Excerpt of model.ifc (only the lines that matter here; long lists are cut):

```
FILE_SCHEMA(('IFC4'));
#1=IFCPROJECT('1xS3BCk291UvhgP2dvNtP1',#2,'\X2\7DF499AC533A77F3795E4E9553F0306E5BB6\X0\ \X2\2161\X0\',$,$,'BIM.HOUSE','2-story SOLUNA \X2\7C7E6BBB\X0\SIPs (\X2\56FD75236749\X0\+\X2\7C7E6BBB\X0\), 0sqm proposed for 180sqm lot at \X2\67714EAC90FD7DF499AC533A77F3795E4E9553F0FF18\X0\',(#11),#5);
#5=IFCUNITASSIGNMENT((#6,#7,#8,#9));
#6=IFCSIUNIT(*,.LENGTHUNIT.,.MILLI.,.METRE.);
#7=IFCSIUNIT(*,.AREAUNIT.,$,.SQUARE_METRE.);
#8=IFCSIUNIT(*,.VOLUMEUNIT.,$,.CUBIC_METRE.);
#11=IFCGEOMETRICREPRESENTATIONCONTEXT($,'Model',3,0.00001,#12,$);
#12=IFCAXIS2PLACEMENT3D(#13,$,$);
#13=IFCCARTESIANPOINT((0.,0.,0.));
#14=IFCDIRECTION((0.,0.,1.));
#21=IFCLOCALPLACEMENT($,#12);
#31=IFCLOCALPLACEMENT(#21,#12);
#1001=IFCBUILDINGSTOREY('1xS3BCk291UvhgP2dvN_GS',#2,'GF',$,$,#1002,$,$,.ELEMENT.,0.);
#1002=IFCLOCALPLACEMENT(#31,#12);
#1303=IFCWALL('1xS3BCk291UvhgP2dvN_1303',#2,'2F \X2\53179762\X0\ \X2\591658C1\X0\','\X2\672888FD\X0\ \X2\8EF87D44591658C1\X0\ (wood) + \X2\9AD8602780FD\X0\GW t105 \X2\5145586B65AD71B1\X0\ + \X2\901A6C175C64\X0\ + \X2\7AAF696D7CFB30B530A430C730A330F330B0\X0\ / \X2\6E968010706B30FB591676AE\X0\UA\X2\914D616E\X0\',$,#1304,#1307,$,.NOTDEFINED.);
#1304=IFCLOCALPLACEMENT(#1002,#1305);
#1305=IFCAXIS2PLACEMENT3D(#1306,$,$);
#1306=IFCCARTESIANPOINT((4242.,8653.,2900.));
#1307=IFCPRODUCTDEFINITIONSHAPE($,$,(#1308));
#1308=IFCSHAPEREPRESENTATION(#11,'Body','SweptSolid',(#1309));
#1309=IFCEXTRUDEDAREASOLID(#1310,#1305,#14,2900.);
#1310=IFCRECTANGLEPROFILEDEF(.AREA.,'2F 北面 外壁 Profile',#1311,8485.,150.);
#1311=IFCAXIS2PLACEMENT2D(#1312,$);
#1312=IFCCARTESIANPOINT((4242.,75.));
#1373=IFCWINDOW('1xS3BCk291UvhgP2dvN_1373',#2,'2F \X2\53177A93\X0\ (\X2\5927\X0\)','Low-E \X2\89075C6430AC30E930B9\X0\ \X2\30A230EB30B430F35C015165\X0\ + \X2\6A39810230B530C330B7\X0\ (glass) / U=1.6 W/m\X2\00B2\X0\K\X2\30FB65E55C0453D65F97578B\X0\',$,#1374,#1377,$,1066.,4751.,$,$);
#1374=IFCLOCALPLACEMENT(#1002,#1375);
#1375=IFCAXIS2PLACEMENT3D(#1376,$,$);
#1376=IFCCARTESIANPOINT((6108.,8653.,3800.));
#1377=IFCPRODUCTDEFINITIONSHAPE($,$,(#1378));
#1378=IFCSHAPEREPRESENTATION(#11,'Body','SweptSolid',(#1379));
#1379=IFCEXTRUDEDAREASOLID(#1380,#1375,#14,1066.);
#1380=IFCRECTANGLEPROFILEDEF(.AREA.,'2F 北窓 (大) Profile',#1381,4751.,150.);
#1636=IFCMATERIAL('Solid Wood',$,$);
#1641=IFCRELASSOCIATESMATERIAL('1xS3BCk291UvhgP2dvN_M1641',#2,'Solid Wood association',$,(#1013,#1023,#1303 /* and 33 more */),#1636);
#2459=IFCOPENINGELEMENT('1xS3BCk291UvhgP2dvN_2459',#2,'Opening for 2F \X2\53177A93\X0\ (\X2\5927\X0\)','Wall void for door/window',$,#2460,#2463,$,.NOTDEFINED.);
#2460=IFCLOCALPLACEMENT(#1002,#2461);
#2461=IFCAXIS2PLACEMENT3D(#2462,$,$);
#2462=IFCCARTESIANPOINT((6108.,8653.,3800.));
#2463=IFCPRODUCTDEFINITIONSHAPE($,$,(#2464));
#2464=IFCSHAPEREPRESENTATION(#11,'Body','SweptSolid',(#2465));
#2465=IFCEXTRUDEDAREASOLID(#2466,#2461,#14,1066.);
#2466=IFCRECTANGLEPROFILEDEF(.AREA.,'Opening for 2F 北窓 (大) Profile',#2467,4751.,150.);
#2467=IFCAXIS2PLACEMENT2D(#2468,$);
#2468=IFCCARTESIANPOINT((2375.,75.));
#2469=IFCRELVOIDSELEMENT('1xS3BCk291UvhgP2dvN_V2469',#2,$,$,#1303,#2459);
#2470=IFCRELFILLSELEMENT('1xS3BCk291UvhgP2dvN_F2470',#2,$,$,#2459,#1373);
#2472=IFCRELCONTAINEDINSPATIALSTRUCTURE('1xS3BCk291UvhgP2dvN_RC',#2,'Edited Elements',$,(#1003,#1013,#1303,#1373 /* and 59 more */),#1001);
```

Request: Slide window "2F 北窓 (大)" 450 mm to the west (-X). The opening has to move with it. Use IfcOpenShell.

```python
import ifcopenshell
import ifcopenshell.api.geometry
import ifcopenshell.util.placement
import ifcopenshell.util.unit

model = ifcopenshell.open("model.ifc")
unit_scale = ifcopenshell.util.unit.calculate_unit_scale(model)

window = model.by_guid("1xS3BCk291UvhgP2dvN_1373")
opening = window.FillsVoids[0].RelatingOpeningElement
wall = opening.VoidsElements[0].RelatingBuildingElement

wall_matrix = ifcopenshell.util.placement.get_local_placement(wall.ObjectPlacement)
shift = wall_matrix[:3, 0] * -0.45 / unit_scale
before = ifcopenshell.util.placement.get_local_placement(window.ObjectPlacement)[:3, 3].copy()

# The window is not placed relative to its opening, so move both.
for product in (opening, window):
    matrix = ifcopenshell.util.placement.get_local_placement(product.ObjectPlacement)
    matrix[:3, 3] += shift
    ifcopenshell.api.geometry.edit_object_placement(model, product=product, matrix=matrix, is_si=False)

after = ifcopenshell.util.placement.get_local_placement(window.ObjectPlacement)[:3, 3]
print("window moved by", (after - before).round(3) + 0.0)

model.write("model_edited.ifc")
```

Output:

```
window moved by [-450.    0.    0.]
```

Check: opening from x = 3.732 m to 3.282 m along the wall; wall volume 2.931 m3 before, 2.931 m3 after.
